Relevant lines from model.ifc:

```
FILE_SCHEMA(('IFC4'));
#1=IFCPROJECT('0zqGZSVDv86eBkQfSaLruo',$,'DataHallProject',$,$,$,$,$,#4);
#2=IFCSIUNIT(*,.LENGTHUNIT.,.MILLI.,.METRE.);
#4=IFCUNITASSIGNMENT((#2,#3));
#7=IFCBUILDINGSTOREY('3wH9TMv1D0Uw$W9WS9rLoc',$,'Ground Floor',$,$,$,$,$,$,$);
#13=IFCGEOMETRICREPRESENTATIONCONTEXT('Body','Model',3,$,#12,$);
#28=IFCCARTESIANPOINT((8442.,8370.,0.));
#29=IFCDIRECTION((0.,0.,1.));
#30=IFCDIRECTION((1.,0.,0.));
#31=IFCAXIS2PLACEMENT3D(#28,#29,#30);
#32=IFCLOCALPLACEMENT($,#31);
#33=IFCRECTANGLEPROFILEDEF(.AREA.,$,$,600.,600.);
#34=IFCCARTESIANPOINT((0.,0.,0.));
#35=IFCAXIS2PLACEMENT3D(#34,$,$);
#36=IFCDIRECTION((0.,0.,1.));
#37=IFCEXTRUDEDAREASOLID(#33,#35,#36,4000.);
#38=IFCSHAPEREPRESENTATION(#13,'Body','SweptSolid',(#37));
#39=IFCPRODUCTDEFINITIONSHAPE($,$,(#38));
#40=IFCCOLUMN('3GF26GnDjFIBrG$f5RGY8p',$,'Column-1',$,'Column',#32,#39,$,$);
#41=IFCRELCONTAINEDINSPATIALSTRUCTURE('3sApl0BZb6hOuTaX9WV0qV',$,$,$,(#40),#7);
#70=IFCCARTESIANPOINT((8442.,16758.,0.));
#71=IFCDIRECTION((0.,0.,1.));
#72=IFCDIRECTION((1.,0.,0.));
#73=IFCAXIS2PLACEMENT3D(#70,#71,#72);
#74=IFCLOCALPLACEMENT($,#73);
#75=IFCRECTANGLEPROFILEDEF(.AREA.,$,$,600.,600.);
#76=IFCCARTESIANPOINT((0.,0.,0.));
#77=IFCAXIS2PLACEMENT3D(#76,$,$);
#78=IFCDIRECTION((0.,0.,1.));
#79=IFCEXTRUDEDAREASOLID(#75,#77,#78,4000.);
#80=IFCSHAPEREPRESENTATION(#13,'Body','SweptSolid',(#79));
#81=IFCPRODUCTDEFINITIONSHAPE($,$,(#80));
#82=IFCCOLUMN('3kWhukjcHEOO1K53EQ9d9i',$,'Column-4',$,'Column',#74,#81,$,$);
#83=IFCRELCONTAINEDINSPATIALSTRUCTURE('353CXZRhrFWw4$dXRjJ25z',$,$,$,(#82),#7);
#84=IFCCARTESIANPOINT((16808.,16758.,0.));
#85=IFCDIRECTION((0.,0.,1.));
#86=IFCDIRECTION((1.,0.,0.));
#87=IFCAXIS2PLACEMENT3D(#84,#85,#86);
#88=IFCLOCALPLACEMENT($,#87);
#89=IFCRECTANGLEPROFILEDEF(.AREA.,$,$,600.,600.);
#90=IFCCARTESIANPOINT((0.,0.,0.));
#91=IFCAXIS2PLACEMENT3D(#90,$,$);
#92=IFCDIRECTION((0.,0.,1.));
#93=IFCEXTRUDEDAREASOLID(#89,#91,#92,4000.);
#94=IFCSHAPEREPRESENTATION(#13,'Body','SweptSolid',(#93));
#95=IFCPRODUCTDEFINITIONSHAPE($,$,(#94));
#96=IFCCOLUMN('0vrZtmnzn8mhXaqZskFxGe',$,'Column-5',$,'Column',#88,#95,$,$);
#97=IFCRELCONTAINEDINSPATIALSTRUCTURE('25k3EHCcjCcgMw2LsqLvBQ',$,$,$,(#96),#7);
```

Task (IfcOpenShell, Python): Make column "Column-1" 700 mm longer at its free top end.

```python
import ifcopenshell
import ifcopenshell.util.unit

model = ifcopenshell.open("model.ifc")
unit_scale = ifcopenshell.util.unit.calculate_unit_scale(model)

member = model.by_id(40)
change = 0.7 / unit_scale

# The extrusion runs towards the end named, so only its depth changes.
body = next(r for r in member.Representation.Representations if r.RepresentationIdentifier == "Body")
solid = body.Items[0]
old_length = solid.Depth
solid.Depth += change

print(f"length {old_length:g} -> {solid.Depth:g}")

model.write("model_edited.ifc")
```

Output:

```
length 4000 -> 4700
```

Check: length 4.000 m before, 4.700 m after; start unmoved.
